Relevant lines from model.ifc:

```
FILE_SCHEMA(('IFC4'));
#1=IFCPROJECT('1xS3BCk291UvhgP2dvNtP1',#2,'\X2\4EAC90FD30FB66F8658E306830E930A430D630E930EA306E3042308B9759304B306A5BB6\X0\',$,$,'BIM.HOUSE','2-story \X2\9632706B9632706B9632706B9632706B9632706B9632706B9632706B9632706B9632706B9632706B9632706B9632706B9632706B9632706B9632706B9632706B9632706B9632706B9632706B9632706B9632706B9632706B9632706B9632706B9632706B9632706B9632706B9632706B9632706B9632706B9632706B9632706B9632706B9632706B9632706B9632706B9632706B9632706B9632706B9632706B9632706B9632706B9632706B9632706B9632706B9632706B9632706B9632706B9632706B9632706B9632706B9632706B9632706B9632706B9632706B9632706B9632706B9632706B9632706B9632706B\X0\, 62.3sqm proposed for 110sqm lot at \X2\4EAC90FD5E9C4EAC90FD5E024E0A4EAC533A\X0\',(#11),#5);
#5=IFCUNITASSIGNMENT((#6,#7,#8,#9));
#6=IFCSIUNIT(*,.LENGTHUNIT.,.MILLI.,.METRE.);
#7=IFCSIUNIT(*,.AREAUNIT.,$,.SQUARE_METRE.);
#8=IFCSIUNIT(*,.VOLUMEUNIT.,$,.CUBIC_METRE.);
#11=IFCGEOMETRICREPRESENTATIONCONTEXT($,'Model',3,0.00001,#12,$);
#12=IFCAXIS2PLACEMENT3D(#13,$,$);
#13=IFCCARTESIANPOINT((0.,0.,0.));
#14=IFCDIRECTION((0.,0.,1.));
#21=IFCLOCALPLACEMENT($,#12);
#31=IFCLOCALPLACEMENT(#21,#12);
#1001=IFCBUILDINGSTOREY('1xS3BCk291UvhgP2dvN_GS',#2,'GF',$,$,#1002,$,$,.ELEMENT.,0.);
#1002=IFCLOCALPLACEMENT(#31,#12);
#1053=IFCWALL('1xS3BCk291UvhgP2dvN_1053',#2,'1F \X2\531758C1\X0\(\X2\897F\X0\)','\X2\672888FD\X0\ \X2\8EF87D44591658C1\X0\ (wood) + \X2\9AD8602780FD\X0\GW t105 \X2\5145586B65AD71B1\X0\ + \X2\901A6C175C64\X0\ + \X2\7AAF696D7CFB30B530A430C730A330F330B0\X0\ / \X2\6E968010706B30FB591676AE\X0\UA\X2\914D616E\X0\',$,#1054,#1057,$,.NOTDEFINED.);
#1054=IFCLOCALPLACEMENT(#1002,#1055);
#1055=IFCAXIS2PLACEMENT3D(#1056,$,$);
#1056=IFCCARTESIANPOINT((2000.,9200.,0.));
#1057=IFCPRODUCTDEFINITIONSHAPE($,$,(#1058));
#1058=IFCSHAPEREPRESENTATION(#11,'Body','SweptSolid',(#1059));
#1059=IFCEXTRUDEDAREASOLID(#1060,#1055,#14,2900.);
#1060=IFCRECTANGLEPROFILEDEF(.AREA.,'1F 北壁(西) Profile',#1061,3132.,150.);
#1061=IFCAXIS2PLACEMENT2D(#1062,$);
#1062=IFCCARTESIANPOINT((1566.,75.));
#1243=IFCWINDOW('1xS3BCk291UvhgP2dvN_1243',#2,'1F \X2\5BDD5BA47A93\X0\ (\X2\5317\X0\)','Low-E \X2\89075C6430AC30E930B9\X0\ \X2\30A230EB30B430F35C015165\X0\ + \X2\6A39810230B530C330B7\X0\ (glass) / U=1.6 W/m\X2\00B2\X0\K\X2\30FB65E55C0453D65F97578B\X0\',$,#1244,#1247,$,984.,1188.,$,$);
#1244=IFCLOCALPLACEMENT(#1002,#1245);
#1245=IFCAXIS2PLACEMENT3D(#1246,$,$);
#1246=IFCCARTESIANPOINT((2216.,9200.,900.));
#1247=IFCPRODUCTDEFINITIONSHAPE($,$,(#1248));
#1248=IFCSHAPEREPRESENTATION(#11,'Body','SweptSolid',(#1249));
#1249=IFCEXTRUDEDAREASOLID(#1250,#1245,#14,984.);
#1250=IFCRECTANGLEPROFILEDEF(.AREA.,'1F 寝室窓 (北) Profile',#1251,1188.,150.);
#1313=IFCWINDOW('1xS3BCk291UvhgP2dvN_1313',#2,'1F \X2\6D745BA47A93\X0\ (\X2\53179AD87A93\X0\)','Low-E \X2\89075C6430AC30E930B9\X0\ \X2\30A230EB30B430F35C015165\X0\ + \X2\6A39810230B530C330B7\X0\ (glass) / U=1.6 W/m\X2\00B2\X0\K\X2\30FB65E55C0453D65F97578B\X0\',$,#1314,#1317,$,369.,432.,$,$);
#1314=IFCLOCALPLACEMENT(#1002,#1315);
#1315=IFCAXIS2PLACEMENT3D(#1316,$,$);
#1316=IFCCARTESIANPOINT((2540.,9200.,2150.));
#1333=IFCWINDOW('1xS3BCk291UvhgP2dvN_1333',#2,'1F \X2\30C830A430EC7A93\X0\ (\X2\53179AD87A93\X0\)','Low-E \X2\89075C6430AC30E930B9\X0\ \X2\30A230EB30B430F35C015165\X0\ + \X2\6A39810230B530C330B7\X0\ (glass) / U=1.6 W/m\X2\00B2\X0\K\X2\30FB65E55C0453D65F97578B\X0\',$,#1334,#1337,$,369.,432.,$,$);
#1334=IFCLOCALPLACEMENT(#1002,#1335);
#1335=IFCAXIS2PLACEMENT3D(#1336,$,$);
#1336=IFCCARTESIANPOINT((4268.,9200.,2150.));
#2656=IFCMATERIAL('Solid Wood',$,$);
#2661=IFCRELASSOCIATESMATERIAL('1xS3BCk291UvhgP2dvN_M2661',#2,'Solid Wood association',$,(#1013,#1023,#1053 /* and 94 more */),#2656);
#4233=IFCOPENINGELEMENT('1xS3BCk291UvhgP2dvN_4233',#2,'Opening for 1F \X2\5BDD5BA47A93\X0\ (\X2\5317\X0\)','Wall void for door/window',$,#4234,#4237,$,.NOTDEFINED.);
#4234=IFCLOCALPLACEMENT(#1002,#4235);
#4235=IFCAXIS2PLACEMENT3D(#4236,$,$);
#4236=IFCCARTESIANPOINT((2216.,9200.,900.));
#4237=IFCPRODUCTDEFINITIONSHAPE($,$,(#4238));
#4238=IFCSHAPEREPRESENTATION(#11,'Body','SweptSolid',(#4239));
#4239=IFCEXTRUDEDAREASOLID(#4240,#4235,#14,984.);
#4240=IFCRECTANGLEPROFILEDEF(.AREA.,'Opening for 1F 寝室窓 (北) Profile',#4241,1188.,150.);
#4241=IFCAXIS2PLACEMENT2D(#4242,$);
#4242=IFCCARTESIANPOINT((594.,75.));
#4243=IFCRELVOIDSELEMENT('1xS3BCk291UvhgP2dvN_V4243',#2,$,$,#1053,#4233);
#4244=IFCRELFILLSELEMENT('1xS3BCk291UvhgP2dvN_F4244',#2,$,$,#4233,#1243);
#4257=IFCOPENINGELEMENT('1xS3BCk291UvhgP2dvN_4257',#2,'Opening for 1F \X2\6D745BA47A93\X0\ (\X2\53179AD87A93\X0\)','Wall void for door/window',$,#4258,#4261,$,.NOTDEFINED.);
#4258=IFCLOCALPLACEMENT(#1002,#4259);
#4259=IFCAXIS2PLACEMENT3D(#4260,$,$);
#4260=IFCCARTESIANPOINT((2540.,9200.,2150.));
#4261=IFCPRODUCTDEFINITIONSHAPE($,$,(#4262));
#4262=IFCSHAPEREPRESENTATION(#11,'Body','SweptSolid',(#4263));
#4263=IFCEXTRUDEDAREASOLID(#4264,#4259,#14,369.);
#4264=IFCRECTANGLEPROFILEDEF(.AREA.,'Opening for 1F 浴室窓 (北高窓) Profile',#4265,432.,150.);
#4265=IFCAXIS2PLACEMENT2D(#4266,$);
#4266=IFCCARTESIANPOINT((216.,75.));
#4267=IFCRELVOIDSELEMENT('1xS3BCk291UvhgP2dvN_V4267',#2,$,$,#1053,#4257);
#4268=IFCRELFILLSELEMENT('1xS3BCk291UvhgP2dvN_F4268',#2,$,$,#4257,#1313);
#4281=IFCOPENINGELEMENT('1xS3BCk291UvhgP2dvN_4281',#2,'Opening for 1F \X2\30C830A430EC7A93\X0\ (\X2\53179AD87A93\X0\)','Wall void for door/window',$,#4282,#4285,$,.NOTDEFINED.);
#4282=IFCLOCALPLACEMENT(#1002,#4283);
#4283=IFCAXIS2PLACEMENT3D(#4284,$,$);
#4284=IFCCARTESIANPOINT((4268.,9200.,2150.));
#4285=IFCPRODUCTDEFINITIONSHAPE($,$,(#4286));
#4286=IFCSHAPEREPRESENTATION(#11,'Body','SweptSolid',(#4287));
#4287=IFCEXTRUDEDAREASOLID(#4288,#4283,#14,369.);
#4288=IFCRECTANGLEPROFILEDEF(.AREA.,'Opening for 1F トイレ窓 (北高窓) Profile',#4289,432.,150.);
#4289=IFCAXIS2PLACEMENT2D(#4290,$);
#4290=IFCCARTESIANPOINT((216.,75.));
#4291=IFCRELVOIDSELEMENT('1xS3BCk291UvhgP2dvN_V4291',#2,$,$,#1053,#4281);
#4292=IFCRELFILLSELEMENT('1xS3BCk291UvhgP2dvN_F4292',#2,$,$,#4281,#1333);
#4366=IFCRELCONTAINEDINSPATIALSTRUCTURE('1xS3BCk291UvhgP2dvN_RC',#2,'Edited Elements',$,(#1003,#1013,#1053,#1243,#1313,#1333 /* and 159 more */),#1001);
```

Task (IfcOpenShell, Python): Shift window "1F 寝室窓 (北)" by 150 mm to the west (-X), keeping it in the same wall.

```python
import ifcopenshell
import ifcopenshell.api.geometry
import ifcopenshell.util.placement
import ifcopenshell.util.unit

model = ifcopenshell.open("model.ifc")
unit_scale = ifcopenshell.util.unit.calculate_unit_scale(model)

window = model.by_guid("1xS3BCk291UvhgP2dvN_1243")
opening = window.FillsVoids[0].RelatingOpeningElement
wall = opening.VoidsElements[0].RelatingBuildingElement

wall_matrix = ifcopenshell.util.placement.get_local_placement(wall.ObjectPlacement)
shift = wall_matrix[:3, 0] * -0.15 / unit_scale
before = ifcopenshell.util.placement.get_local_placement(window.ObjectPlacement)[:3, 3].copy()

# The window is not placed relative to its opening, so move both.
for product in (opening, window):
    matrix = ifcopenshell.util.placement.get_local_placement(product.ObjectPlacement)
    matrix[:3, 3] += shift
    ifcopenshell.api.geometry.edit_object_placement(model, product=product, matrix=matrix, is_si=False)

after = ifcopenshell.util.placement.get_local_placement(window.ObjectPlacement)[:3, 3]
print("window moved by", (after - before).round(3) + 0.0)

model.write("model_rev.ifc")
```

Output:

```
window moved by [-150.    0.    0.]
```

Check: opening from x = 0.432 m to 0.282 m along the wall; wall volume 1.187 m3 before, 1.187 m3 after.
